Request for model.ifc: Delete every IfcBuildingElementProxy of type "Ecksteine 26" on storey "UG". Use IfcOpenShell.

First a look at what the model holds.

```python
import ifcopenshell
import ifcopenshell.util.element

model = ifcopenshell.open("model.ifc")
print(model.schema)
storey = next(s for s in model.by_type("IfcBuildingStorey") if s.Name == "UG")
proxies = [e for e in ifcopenshell.util.element.get_decomposition(storey) if e.is_a("IfcBuildingElementProxy")]
seen = {}
for e in proxies:
    element_type = ifcopenshell.util.element.get_type(e)
    name = element_type.Name if element_type not in (None, e) else None
    seen[name] = seen.get(name, 0) + 1
for name, count in sorted(seen.items(), key=str):
    print(count, "x", name)
```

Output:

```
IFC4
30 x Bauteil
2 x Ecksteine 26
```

```python
import ifcopenshell
import ifcopenshell.api.root
import ifcopenshell.util.element

model = ifcopenshell.open("model.ifc")

storey = next(s for s in model.by_type("IfcBuildingStorey") if s.Name == "UG")
proxies = [e for e in ifcopenshell.util.element.get_decomposition(storey) if e.is_a("IfcBuildingElementProxy")]
targets = [e for e in proxies if (t := ifcopenshell.util.element.get_type(e)) not in (None, e) and t.Name == "Ecksteine 26"]

for e in targets:
    ifcopenshell.api.root.remove_product(model, product=e)
print(len(targets), "removed")

model.write("model_rev.ifc")
```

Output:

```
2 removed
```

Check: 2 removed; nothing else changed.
